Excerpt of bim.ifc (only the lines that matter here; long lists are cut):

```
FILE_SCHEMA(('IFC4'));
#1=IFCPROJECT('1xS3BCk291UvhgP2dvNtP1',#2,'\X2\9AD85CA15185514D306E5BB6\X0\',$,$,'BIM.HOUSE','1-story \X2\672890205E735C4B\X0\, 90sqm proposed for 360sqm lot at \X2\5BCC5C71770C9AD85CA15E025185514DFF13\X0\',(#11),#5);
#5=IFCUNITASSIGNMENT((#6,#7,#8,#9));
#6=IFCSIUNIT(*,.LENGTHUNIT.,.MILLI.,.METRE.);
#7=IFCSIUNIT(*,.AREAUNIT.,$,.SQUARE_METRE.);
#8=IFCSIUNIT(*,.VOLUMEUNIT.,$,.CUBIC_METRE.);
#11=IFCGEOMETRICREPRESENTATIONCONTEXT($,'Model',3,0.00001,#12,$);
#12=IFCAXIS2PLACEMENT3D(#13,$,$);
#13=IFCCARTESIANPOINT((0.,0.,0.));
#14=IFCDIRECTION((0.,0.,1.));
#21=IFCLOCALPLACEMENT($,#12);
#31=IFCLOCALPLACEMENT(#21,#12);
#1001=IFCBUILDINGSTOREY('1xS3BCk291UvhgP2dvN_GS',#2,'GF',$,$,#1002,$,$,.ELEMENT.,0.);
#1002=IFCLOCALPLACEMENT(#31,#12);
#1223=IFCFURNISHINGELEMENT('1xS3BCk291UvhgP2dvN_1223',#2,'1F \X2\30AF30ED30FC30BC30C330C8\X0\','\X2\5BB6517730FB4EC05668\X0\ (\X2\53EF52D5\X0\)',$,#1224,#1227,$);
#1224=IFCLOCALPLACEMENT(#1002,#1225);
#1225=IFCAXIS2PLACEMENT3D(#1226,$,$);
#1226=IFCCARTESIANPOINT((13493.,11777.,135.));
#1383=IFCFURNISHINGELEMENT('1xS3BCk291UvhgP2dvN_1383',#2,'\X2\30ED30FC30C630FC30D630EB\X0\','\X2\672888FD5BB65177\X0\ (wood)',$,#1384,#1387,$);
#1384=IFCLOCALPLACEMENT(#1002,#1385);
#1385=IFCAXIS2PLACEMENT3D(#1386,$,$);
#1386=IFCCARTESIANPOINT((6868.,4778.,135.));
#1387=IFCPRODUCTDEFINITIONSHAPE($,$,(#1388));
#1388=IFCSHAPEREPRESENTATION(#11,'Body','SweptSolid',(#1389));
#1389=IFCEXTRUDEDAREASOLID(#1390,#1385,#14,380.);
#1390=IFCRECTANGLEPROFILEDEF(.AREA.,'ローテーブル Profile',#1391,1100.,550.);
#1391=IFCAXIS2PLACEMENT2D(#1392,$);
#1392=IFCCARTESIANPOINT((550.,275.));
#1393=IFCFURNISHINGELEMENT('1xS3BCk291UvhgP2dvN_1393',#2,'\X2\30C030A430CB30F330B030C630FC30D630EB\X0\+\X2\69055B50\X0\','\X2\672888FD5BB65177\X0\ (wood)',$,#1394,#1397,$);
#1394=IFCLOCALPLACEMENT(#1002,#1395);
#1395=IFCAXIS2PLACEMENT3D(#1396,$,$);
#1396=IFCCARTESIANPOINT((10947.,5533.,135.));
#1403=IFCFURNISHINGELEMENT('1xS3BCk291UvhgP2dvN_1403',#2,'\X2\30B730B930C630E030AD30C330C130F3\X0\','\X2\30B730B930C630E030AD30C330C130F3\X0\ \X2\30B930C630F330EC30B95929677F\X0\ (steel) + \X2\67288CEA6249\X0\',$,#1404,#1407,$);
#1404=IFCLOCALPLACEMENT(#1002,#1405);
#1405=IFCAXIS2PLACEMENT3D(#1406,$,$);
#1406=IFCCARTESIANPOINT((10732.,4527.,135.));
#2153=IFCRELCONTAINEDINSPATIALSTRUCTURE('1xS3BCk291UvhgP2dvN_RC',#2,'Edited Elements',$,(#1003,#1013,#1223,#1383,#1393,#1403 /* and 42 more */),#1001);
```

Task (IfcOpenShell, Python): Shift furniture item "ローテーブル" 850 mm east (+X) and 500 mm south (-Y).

```python
import ifcopenshell
import ifcopenshell.api.geometry
import ifcopenshell.util.placement
import ifcopenshell.util.unit

model = ifcopenshell.open("bim.ifc")
unit_scale = ifcopenshell.util.unit.calculate_unit_scale(model)

item = model.by_id(1383)
matrix = ifcopenshell.util.placement.get_local_placement(item.ObjectPlacement)
matrix[0, 3] += 0.85 / unit_scale
matrix[1, 3] -= 0.5 / unit_scale
ifcopenshell.api.geometry.edit_object_placement(model, product=item, matrix=matrix, is_si=False)

print(ifcopenshell.util.placement.get_local_placement(item.ObjectPlacement).round(3) + 0.0)

model.write("bim_updated.ifc")
```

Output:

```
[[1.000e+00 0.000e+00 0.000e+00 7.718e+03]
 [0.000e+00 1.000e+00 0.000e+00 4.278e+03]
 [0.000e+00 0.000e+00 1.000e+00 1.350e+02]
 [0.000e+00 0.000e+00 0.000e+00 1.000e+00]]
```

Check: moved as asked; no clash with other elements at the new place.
